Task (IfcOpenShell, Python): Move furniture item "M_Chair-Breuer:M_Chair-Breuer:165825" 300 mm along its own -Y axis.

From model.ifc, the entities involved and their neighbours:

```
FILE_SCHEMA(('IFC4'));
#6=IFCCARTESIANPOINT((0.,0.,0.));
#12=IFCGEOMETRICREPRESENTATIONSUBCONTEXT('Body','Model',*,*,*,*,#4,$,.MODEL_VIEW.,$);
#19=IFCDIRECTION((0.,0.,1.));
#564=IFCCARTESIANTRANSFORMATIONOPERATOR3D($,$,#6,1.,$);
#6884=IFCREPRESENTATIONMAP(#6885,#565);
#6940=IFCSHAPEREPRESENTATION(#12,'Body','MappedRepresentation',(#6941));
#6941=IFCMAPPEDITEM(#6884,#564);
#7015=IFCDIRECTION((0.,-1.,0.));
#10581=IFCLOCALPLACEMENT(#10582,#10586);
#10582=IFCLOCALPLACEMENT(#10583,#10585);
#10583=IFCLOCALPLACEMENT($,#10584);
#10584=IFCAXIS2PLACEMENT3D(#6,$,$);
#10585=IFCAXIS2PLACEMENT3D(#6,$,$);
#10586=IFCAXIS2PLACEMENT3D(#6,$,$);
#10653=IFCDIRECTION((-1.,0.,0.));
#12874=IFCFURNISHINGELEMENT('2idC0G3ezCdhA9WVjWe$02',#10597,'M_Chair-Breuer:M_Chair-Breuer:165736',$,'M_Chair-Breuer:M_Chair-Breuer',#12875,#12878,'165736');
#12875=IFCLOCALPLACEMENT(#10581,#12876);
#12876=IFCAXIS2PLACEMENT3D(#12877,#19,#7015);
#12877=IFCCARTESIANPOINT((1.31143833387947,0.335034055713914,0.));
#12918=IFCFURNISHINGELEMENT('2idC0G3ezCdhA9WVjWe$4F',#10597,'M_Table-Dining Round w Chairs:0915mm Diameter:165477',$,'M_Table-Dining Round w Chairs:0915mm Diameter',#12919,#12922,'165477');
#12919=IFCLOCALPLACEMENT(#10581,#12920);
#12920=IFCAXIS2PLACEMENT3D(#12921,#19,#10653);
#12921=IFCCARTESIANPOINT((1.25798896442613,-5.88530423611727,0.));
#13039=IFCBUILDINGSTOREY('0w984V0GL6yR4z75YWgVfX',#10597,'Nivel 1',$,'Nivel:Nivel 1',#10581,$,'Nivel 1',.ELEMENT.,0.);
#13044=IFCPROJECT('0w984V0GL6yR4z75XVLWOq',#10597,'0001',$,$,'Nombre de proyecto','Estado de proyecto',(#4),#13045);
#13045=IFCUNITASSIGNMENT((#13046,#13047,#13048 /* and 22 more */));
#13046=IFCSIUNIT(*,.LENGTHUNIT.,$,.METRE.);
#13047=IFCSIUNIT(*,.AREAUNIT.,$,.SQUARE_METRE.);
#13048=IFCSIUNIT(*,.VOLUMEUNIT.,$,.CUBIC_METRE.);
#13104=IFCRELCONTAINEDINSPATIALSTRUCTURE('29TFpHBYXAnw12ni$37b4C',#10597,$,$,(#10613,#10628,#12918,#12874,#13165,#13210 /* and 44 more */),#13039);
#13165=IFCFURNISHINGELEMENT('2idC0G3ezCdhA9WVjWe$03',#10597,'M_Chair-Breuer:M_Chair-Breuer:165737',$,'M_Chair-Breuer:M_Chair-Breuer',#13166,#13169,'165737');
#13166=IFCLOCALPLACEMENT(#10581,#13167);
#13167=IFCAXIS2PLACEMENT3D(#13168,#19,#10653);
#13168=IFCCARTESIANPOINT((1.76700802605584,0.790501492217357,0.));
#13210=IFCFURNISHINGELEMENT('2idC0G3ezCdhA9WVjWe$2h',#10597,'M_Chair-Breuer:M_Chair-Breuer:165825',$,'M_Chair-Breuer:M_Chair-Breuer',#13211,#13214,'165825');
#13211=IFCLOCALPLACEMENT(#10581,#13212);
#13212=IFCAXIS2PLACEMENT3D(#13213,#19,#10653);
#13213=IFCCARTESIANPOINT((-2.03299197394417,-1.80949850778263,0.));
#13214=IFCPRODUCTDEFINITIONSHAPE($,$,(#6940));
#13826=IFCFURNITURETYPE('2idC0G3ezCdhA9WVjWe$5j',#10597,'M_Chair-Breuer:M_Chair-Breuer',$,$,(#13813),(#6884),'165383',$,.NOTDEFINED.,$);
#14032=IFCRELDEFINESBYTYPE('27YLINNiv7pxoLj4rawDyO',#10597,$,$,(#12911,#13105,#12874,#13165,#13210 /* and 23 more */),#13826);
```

```python
import ifcopenshell
import ifcopenshell.api.geometry
import ifcopenshell.util.placement

model = ifcopenshell.open("model.ifc")

item = model.by_guid("2idC0G3ezCdhA9WVjWe$2h")
matrix = ifcopenshell.util.placement.get_local_placement(item.ObjectPlacement)
matrix[:3, 3] -= matrix[:3, 1] * 0.3
ifcopenshell.api.geometry.edit_object_placement(model, product=item, matrix=matrix, is_si=False)

print(ifcopenshell.util.placement.get_local_placement(item.ObjectPlacement).round(3) + 0.0)

model.write("model_edited.ifc")
```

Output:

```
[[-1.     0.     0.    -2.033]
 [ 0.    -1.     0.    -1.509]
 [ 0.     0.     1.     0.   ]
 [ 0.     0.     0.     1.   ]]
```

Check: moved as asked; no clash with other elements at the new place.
